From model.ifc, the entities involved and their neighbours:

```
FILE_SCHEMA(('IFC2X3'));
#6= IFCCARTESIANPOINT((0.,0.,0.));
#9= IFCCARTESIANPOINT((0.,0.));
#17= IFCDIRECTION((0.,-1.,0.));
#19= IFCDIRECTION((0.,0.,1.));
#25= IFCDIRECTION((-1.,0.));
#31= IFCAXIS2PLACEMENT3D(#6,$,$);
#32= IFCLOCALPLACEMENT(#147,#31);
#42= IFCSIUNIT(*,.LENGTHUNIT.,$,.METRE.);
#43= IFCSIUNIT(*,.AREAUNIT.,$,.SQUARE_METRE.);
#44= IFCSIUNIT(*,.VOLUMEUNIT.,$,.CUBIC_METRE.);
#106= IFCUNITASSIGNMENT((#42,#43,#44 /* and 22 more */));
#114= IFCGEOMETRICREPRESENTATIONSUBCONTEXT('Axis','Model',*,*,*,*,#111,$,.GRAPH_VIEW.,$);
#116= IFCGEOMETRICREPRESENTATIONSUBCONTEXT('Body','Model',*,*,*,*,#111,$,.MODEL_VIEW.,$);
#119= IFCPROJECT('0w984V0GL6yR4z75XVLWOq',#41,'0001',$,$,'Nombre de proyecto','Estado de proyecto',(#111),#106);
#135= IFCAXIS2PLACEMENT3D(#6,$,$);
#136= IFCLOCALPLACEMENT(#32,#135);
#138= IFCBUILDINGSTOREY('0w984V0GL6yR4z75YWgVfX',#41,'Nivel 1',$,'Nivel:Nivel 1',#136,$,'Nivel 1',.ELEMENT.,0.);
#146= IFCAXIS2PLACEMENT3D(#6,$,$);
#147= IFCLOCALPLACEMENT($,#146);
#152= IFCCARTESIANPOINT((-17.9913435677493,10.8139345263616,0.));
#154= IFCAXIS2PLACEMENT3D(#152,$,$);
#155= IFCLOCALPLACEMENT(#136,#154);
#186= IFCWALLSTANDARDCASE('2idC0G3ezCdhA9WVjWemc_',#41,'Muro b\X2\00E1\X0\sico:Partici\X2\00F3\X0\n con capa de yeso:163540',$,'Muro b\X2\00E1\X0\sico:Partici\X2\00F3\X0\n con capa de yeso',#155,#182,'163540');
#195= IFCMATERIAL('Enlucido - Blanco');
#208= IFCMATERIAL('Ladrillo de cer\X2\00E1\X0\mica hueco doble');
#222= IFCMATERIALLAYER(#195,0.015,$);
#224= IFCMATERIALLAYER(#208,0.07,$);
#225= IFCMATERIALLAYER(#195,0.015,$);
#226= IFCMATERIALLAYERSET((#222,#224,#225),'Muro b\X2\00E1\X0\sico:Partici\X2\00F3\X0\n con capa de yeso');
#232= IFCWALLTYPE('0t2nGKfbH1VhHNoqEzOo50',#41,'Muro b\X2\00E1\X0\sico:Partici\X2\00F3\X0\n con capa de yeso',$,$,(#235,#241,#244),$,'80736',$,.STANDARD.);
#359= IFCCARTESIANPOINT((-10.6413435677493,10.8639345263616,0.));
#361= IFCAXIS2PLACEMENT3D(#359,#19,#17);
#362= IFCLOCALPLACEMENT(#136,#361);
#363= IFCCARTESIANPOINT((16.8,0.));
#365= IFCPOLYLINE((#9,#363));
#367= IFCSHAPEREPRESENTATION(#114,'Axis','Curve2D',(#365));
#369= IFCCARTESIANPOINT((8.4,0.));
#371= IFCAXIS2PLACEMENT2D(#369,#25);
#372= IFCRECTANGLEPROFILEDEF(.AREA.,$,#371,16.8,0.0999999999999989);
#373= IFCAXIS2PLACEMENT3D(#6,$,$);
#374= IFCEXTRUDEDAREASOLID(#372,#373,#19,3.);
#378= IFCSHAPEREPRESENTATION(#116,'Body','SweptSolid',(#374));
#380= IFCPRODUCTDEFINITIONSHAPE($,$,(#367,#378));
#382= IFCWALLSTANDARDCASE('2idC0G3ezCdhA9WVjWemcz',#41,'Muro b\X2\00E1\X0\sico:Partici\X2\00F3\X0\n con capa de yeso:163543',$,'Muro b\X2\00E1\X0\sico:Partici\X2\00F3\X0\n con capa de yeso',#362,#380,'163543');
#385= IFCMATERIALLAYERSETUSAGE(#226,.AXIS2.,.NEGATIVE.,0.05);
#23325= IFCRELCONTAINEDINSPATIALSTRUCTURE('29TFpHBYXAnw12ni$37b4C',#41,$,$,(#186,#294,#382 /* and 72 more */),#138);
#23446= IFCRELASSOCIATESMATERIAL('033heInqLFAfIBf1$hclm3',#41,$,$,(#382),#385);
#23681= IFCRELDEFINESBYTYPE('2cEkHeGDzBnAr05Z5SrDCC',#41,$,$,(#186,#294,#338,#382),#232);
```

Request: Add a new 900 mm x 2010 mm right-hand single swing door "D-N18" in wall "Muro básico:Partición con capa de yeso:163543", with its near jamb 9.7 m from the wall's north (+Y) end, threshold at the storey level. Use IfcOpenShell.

```python
import numpy as np
import ifcopenshell
import ifcopenshell.api.feature
import ifcopenshell.api.geometry
import ifcopenshell.api.root
import ifcopenshell.api.spatial
import ifcopenshell.api.type
import ifcopenshell.geom
import ifcopenshell.util.element
import ifcopenshell.util.placement
import ifcopenshell.util.representation
import ifcopenshell.util.shape
import ifcopenshell.util.unit

model = ifcopenshell.open("model.ifc")
unit_scale = ifcopenshell.util.unit.calculate_unit_scale(model)
settings = ifcopenshell.geom.settings()


def volume(element):
    """Net volume in cubic metres, openings subtracted."""
    shape = ifcopenshell.geom.create_shape(settings, element)
    return ifcopenshell.util.shape.get_volume(shape.geometry)


wall = model.by_guid("2idC0G3ezCdhA9WVjWemcz")
storey = ifcopenshell.util.element.get_container(wall, ifc_class="IfcBuildingStorey")
context = ifcopenshell.util.representation.get_context(model, "Model", "Body", "MODEL_VIEW")
before = volume(wall)

width, height, from_end, sill = 0.9, 2.01, 9.7, 0.0  # metres

# The wall runs along its own X axis, and the end named is its -X end.
wall_shape = ifcopenshell.geom.create_shape(settings, wall)
x, y, z = ifcopenshell.util.shape.get_vertices(wall_shape.geometry).T
start = x.min() + from_end
face, thickness = float(y.min()), float(y.max() - y.min())
wall_matrix = ifcopenshell.util.placement.get_local_placement(wall.ObjectPlacement)
level = ifcopenshell.util.placement.get_local_placement(storey.ObjectPlacement)[2, 3]


def in_wall(x, y):
    """Placement at x, y metres in the wall's axes, at sill height."""
    matrix = wall_matrix.copy()
    matrix[:, 3] = wall_matrix @ np.array([x / unit_scale, y / unit_scale, 0.0, 1.0])
    matrix[2, 3] = level + sill / unit_scale
    return matrix


# Opening: a box that overshoots both wall faces by 50 mm.
opening = ifcopenshell.api.root.create_entity(model, ifc_class="IfcOpeningElement")
box = ifcopenshell.api.geometry.add_wall_representation(
    model, context=context, length=width, height=height, thickness=thickness + 0.1
)
ifcopenshell.api.geometry.assign_representation(model, product=opening, representation=box)
ifcopenshell.api.geometry.edit_object_placement(model, product=opening, matrix=in_wall(start, face - 0.05), is_si=False)
ifcopenshell.api.feature.add_feature(model, feature=opening, element=wall)

door = ifcopenshell.api.root.create_entity(model, ifc_class="IfcDoor", name="D-N18")
door.OverallWidth, door.OverallHeight = width / unit_scale, height / unit_scale
body = ifcopenshell.api.geometry.add_door_representation(
    model,
    context=context,
    overall_width=door.OverallWidth,
    overall_height=door.OverallHeight,
    operation_type="SINGLE_SWING_RIGHT",
    lining_properties={"LiningDepth": thickness / unit_scale, "ThresholdDepth": thickness / unit_scale},
)
ifcopenshell.api.geometry.assign_representation(model, product=door, representation=body)
ifcopenshell.api.spatial.assign_container(model, products=[door], relating_structure=storey)
fills = ifcopenshell.api.feature.add_filling(model, opening=opening, element=door)
fills.OwnerHistory = door.OwnerHistory  # required in IFC2X3

# IFC2X3 keeps the operation on the door style.
style = ifcopenshell.api.root.create_entity(model, ifc_class="IfcDoorStyle", name="D-N18")
style.OperationType, style.ConstructionType = "SINGLE_SWING_RIGHT", "NOTDEFINED"
style.ParameterTakesPrecedence = style.Sizeable = False
ifcopenshell.api.type.assign_type(model, related_objects=[door], relating_type=style)

# The lining spans the wall, so the door starts at the wall face.
ifcopenshell.api.geometry.edit_object_placement(model, product=door, matrix=in_wall(start, face), is_si=False)

after = volume(wall)

print(f"wall volume {before:.3f} -> {after:.3f} m3")

model.write("model_rev.ifc")
```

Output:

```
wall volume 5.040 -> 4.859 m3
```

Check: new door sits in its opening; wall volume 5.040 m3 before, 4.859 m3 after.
